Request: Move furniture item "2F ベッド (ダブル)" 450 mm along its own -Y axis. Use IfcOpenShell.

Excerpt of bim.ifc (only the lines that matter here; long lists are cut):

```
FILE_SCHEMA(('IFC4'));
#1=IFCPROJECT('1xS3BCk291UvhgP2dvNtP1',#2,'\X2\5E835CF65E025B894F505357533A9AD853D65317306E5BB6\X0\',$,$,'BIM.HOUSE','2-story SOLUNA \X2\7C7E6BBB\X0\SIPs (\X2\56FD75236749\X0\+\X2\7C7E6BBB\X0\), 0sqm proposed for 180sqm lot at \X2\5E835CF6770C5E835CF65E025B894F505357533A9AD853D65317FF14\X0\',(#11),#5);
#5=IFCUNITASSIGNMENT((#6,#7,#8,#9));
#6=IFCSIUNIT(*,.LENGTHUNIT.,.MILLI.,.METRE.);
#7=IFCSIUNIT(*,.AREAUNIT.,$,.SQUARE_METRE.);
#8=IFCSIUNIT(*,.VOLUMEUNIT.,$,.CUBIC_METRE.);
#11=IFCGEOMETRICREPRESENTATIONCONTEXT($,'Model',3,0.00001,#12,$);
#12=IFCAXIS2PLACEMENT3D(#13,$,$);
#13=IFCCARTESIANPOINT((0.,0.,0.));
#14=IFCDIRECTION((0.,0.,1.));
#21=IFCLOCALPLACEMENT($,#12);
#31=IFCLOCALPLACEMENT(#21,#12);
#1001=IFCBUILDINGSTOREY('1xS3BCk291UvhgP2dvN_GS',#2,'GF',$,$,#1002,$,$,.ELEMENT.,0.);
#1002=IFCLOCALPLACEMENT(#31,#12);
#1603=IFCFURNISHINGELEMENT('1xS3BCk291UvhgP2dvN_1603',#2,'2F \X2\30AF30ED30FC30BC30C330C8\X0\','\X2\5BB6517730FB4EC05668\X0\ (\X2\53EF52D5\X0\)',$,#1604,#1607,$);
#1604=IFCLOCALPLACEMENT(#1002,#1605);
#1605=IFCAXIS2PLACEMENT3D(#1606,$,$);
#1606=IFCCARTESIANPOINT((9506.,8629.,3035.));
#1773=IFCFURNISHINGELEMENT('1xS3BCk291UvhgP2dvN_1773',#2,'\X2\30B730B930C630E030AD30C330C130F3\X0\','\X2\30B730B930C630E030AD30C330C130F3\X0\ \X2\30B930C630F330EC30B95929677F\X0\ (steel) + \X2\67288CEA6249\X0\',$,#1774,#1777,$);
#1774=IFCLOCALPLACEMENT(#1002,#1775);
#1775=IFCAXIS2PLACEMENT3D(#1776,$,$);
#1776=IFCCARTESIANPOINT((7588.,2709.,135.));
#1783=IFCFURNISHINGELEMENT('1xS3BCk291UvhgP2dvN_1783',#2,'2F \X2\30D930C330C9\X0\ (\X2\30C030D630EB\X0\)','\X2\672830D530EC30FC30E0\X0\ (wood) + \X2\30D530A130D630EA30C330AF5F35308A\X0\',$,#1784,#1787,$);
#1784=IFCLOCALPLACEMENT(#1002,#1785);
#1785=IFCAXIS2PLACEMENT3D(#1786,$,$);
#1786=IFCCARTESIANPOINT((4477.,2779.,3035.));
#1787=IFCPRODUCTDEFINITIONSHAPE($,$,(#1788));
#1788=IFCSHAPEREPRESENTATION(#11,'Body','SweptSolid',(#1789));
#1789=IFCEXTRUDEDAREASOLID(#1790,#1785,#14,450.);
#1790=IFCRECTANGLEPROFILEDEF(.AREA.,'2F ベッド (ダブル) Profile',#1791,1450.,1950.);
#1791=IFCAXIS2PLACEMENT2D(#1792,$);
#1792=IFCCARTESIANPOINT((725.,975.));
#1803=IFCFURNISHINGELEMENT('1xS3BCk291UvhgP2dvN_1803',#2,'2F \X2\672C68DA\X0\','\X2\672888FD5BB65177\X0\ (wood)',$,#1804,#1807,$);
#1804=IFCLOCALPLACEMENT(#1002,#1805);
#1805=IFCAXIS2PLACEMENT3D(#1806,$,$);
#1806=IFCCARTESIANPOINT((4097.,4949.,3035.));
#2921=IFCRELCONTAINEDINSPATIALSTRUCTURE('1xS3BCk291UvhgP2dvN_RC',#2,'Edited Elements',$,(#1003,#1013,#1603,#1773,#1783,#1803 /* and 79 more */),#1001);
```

```python
import ifcopenshell
import ifcopenshell.api.geometry
import ifcopenshell.util.placement

model = ifcopenshell.open("bim.ifc")

item = model.by_guid("1xS3BCk291UvhgP2dvN_1783")
matrix = ifcopenshell.util.placement.get_local_placement(item.ObjectPlacement)
matrix[:3, 3] -= matrix[:3, 1] * 450.0
ifcopenshell.api.geometry.edit_object_placement(model, product=item, matrix=matrix, is_si=False)

print(ifcopenshell.util.placement.get_local_placement(item.ObjectPlacement).round(3) + 0.0)

model.write("bim_rev.ifc")
```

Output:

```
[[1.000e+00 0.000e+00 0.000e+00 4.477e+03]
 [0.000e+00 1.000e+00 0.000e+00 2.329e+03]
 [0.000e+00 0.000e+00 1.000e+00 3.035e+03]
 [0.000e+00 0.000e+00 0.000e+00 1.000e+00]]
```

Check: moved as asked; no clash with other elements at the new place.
